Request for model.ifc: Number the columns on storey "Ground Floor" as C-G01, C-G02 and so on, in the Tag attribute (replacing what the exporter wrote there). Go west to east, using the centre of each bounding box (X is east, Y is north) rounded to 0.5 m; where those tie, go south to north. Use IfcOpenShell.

First a look at what the model holds.

```python
import ifcopenshell
import ifcopenshell.util.element
import ifcopenshell.util.placement

model = ifcopenshell.open("model.ifc")
print(model.schema)
storey = next(s for s in model.by_type("IfcBuildingStorey") if s.Name == "Ground Floor")
columns = [e for e in ifcopenshell.util.element.get_decomposition(storey) if e.is_a("IfcColumn")]
for e in sorted(columns, key=lambda e: e.id()):
    origin = ifcopenshell.util.placement.get_local_placement(e.ObjectPlacement)[:3, 3]
    print(e.id(), e.Tag, e.Name, origin.round(2) + 0.0, sep=" | ")
```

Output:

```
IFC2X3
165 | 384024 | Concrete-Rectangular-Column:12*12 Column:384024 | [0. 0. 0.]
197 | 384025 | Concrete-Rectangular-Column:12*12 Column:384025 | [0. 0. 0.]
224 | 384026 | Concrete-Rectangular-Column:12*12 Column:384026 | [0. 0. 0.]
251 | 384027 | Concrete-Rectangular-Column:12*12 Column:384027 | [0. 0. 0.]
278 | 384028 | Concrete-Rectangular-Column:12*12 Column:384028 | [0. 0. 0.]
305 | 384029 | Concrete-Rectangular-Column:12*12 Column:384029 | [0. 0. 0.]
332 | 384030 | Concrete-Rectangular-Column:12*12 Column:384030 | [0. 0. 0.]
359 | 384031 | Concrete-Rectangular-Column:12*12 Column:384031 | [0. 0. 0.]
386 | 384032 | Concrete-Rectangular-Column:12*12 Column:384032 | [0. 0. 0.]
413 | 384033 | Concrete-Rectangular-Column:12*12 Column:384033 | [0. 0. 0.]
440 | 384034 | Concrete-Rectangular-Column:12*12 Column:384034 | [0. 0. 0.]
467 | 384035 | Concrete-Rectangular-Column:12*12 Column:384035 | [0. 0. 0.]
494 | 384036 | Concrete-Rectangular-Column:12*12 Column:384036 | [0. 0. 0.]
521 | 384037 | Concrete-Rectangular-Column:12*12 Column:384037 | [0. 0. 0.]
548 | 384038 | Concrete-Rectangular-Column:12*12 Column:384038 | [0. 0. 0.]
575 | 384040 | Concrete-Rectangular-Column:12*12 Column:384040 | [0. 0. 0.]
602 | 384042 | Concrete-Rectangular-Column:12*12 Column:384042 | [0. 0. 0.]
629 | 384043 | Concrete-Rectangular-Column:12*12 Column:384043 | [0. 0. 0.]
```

```python
import ifcopenshell
import ifcopenshell.geom
import ifcopenshell.util.element
import ifcopenshell.util.shape

model = ifcopenshell.open("model.ifc")
settings = ifcopenshell.geom.settings()
settings.set("use-world-coords", True)


def centre(element):
    shape = ifcopenshell.geom.create_shape(settings, element)
    return ifcopenshell.util.shape.get_bbox_centroid(shape.geometry)


storey = next(s for s in model.by_type("IfcBuildingStorey") if s.Name == "Ground Floor")
columns = [e for e in ifcopenshell.util.element.get_decomposition(storey) if e.is_a("IfcColumn")]

# Insertion points can sit at a corner or the storey origin, so sort by the geometry (in metres).
centres = {e: centre(e) for e in columns}
columns.sort(key=lambda e: (round(centres[e][0] / 0.5), centres[e][1]))

for i, e in enumerate(columns, start=1):
    number = f"C-G{i:02d}"
    e.Tag = number
    print(e.id(), number)

model.write("model_edited.ifc")
```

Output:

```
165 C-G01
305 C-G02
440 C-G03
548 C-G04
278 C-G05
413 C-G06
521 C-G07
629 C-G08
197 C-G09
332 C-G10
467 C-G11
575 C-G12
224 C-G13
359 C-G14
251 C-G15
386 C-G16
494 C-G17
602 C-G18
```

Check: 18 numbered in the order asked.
